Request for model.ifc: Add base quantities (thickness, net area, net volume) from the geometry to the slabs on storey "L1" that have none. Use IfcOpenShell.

First a look at what the model holds.

```python
import ifcopenshell
import ifcopenshell.util.element
import ifcopenshell.util.unit

model = ifcopenshell.open("model.ifc")
print(model.schema)
for unit_type in ("LENGTHUNIT", "AREAUNIT", "VOLUMEUNIT"):
    print(unit_type, ifcopenshell.util.unit.calculate_unit_scale(model, unit_type))
storey = next(s for s in model.by_type("IfcBuildingStorey") if s.Name == "L1")
slabs = [e for e in ifcopenshell.util.element.get_decomposition(storey) if e.is_a("IfcSlab")]
for e in sorted(slabs, key=lambda e: e.id()):
    print(e.id(), e.is_a(), e.Name, list(ifcopenshell.util.element.get_psets(e, qtos_only=True)), sep=" | ")
```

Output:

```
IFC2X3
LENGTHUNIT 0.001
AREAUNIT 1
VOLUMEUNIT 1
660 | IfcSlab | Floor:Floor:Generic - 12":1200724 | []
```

```python
import ifcopenshell
import ifcopenshell.api.pset
import ifcopenshell.geom
import ifcopenshell.util.element
import ifcopenshell.util.shape
import ifcopenshell.util.unit

model = ifcopenshell.open("model.ifc")
unit_scale = ifcopenshell.util.unit.calculate_unit_scale(model)
area_scale = ifcopenshell.util.unit.calculate_unit_scale(model, "AREAUNIT")
volume_scale = ifcopenshell.util.unit.calculate_unit_scale(model, "VOLUMEUNIT")
settings = ifcopenshell.geom.settings()

storey = next(s for s in model.by_type("IfcBuildingStorey") if s.Name == "L1")
slabs = [e for e in ifcopenshell.util.element.get_decomposition(storey) if e.is_a("IfcSlab")]

for e in sorted(slabs, key=lambda e: e.id()):
    if ifcopenshell.util.element.get_psets(e, qtos_only=True, should_inherit=False):
        continue
    # Geometry comes back in metres, in the element's own axes.
    shape = ifcopenshell.geom.create_shape(settings, e)
    values = {
        "Width": ifcopenshell.util.shape.get_z(shape.geometry) / unit_scale,
        "NetArea": ifcopenshell.util.shape.get_footprint_area(shape.geometry) / area_scale,
        "NetVolume": ifcopenshell.util.shape.get_volume(shape.geometry) / volume_scale,
    }
    qto = ifcopenshell.api.pset.add_qto(model, product=e, name="BaseQuantities")
    ifcopenshell.api.pset.edit_qto(model, qto=qto, properties=values)
    print(e.id(), {k: round(v, 3) for k, v in values.items()})

model.write("model-out.ifc")
```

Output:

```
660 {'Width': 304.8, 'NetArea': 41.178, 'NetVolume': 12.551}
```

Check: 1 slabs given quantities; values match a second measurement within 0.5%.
